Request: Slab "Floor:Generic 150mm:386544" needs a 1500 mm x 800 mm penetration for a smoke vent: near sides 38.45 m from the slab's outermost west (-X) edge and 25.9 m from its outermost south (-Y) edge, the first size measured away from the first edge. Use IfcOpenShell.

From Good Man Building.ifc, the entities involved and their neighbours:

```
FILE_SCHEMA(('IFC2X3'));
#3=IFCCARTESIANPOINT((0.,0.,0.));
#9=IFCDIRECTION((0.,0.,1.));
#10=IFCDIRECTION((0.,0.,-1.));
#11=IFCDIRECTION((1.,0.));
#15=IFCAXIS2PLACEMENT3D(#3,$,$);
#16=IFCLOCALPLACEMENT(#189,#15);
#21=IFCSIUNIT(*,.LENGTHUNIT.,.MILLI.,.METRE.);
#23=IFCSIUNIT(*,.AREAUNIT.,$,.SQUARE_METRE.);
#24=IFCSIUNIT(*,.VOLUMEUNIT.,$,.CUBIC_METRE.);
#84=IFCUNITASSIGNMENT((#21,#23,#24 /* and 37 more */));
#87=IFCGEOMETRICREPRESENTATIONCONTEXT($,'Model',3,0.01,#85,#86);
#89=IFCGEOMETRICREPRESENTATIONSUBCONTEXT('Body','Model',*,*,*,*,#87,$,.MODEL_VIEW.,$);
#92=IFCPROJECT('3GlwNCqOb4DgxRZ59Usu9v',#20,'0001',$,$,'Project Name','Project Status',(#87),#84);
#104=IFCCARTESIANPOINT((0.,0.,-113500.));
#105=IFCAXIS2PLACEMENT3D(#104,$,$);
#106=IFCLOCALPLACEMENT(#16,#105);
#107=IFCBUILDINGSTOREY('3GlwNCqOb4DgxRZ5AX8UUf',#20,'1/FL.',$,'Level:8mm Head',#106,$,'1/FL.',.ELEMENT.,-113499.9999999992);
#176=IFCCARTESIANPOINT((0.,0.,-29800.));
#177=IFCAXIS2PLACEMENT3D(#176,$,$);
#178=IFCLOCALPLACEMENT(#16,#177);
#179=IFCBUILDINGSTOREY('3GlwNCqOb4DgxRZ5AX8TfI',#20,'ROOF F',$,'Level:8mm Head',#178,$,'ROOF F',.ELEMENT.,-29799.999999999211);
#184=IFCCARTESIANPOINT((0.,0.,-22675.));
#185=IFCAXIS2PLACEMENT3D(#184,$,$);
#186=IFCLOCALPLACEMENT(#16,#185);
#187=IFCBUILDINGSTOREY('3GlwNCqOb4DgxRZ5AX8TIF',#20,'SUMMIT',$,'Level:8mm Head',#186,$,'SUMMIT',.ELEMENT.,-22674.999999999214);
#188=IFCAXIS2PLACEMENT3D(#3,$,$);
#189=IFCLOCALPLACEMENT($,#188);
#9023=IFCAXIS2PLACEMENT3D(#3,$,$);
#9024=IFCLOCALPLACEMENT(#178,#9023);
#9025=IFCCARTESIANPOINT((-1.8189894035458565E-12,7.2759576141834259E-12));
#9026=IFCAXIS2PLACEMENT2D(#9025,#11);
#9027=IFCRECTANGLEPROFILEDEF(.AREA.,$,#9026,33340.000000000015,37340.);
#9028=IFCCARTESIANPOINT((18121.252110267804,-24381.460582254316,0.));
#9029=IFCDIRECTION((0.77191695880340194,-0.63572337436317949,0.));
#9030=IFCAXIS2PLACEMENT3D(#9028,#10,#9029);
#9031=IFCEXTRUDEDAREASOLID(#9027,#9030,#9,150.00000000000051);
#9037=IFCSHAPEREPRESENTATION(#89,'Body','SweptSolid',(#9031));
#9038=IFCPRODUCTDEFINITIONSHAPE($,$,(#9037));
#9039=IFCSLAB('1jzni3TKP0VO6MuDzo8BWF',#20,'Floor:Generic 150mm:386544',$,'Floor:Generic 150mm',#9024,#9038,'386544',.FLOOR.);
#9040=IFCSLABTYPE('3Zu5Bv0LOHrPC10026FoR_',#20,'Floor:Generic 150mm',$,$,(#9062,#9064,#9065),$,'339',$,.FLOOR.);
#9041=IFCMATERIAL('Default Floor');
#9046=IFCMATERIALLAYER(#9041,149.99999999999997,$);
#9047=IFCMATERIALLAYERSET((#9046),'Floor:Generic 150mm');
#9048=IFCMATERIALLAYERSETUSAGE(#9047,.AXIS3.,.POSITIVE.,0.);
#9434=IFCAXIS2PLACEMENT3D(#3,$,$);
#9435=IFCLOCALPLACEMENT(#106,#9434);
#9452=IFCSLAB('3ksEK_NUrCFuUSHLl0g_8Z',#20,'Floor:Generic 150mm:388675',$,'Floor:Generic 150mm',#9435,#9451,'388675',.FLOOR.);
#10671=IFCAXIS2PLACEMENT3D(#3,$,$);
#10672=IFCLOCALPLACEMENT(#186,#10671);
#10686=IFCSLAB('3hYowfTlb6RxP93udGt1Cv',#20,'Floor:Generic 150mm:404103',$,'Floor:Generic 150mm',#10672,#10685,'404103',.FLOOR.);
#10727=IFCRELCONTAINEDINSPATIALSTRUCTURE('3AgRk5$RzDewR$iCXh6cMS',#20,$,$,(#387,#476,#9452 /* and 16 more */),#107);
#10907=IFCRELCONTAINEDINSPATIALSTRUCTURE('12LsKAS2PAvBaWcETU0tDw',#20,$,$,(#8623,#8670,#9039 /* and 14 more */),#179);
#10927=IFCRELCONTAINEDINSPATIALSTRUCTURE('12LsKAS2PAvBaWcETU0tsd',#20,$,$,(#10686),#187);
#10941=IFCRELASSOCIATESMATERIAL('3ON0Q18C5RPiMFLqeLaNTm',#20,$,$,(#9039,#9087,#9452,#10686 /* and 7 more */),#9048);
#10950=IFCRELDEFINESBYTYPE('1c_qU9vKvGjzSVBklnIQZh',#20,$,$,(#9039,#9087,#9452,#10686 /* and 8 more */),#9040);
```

```python
import numpy as np
import ifcopenshell
import ifcopenshell.api.feature
import ifcopenshell.api.geometry
import ifcopenshell.api.root
import ifcopenshell.geom
import ifcopenshell.util.placement
import ifcopenshell.util.representation
import ifcopenshell.util.shape
import ifcopenshell.util.unit

model = ifcopenshell.open("Good Man Building.ifc")
unit_scale = ifcopenshell.util.unit.calculate_unit_scale(model)
settings = ifcopenshell.geom.settings()


def volume(element):
    """Net volume in cubic metres, openings subtracted."""
    shape = ifcopenshell.geom.create_shape(settings, element)
    return ifcopenshell.util.shape.get_volume(shape.geometry)


slab = model.by_guid("1jzni3TKP0VO6MuDzo8BWF")
before = volume(slab)

# Extent in the slab's own axes, in metres. The edges named are its -X and -Y sides.
slab_shape = ifcopenshell.geom.create_shape(settings, slab)
vertices = ifcopenshell.util.shape.get_vertices(slab_shape.geometry)
x_min, y_min, bottom = vertices.min(axis=0)
top = vertices[:, 2].max()

opening = ifcopenshell.api.root.create_entity(model, ifc_class="IfcOpeningElement", name="Smoke vent opening")
context = ifcopenshell.util.representation.get_context(model, "Model", "Body", "MODEL_VIEW")
width, depth = 1.5, 0.8
outline = [(0.0, 0.0), (width, 0.0), (width, depth), (0.0, depth), (0.0, 0.0)]
# Overshoot both faces by 50 mm so the cut is clean.
shape = ifcopenshell.api.geometry.add_slab_representation(
    model, context=context, depth=top - bottom + 0.1, polyline=outline
)
ifcopenshell.api.geometry.assign_representation(model, product=opening, representation=shape)

matrix = ifcopenshell.util.placement.get_local_placement(slab.ObjectPlacement)
matrix[:, 3] = matrix @ np.append(np.array([x_min + 38.45, y_min + 25.9, bottom - 0.05]) / unit_scale, 1.0)
ifcopenshell.api.geometry.edit_object_placement(model, product=opening, matrix=matrix, is_si=False)
ifcopenshell.api.feature.add_feature(model, feature=opening, element=slab)

after = volume(slab)

print(f"slab volume {before:.3f} -> {after:.3f} m3")

model.write("Good Man Building_updated.ifc")
```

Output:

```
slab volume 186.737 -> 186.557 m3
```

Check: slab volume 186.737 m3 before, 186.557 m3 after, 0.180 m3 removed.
